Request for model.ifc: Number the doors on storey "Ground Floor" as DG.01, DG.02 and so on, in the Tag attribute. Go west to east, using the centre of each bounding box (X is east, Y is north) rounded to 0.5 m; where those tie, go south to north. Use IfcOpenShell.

First a look at what the model holds.

```python
import ifcopenshell
import ifcopenshell.util.element
import ifcopenshell.util.placement

model = ifcopenshell.open("model.ifc")
print(model.schema)
storey = next(s for s in model.by_type("IfcBuildingStorey") if s.Name == "Ground Floor")
doors = [e for e in ifcopenshell.util.element.get_decomposition(storey) if e.is_a("IfcDoor")]
for e in sorted(doors, key=lambda e: e.id()):
    origin = ifcopenshell.util.placement.get_local_placement(e.ObjectPlacement)[:3, 3]
    print(e.id(), e.Tag, e.Name, origin.round(2) + 0.0, sep=" | ")
```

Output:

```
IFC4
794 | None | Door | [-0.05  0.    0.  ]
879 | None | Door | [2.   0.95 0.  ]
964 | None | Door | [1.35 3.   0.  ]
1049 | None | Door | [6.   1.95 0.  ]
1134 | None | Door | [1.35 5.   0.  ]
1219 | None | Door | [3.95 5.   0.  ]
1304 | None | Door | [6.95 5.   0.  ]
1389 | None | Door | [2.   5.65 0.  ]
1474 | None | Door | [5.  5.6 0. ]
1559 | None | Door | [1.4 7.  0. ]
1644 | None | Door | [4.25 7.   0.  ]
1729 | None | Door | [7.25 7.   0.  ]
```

```python
import ifcopenshell
import ifcopenshell.geom
import ifcopenshell.util.element
import ifcopenshell.util.shape

model = ifcopenshell.open("model.ifc")
settings = ifcopenshell.geom.settings()
settings.set("use-world-coords", True)


def centre(element):
    shape = ifcopenshell.geom.create_shape(settings, element)
    return ifcopenshell.util.shape.get_bbox_centroid(shape.geometry)


storey = next(s for s in model.by_type("IfcBuildingStorey") if s.Name == "Ground Floor")
doors = [e for e in ifcopenshell.util.element.get_decomposition(storey) if e.is_a("IfcDoor")]

# Insertion points can sit at a corner or the storey origin, so sort by the geometry (in metres).
centres = {e: centre(e) for e in doors}
doors.sort(key=lambda e: (round(centres[e][0] / 0.5), centres[e][1]))

for i, e in enumerate(doors, start=1):
    number = f"DG.{i:02d}"
    e.Tag = number
    print(e.id(), number)

model.write("model_rev.ifc")
```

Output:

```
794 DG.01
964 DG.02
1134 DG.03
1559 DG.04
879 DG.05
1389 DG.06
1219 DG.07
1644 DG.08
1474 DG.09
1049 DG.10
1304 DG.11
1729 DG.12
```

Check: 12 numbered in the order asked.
